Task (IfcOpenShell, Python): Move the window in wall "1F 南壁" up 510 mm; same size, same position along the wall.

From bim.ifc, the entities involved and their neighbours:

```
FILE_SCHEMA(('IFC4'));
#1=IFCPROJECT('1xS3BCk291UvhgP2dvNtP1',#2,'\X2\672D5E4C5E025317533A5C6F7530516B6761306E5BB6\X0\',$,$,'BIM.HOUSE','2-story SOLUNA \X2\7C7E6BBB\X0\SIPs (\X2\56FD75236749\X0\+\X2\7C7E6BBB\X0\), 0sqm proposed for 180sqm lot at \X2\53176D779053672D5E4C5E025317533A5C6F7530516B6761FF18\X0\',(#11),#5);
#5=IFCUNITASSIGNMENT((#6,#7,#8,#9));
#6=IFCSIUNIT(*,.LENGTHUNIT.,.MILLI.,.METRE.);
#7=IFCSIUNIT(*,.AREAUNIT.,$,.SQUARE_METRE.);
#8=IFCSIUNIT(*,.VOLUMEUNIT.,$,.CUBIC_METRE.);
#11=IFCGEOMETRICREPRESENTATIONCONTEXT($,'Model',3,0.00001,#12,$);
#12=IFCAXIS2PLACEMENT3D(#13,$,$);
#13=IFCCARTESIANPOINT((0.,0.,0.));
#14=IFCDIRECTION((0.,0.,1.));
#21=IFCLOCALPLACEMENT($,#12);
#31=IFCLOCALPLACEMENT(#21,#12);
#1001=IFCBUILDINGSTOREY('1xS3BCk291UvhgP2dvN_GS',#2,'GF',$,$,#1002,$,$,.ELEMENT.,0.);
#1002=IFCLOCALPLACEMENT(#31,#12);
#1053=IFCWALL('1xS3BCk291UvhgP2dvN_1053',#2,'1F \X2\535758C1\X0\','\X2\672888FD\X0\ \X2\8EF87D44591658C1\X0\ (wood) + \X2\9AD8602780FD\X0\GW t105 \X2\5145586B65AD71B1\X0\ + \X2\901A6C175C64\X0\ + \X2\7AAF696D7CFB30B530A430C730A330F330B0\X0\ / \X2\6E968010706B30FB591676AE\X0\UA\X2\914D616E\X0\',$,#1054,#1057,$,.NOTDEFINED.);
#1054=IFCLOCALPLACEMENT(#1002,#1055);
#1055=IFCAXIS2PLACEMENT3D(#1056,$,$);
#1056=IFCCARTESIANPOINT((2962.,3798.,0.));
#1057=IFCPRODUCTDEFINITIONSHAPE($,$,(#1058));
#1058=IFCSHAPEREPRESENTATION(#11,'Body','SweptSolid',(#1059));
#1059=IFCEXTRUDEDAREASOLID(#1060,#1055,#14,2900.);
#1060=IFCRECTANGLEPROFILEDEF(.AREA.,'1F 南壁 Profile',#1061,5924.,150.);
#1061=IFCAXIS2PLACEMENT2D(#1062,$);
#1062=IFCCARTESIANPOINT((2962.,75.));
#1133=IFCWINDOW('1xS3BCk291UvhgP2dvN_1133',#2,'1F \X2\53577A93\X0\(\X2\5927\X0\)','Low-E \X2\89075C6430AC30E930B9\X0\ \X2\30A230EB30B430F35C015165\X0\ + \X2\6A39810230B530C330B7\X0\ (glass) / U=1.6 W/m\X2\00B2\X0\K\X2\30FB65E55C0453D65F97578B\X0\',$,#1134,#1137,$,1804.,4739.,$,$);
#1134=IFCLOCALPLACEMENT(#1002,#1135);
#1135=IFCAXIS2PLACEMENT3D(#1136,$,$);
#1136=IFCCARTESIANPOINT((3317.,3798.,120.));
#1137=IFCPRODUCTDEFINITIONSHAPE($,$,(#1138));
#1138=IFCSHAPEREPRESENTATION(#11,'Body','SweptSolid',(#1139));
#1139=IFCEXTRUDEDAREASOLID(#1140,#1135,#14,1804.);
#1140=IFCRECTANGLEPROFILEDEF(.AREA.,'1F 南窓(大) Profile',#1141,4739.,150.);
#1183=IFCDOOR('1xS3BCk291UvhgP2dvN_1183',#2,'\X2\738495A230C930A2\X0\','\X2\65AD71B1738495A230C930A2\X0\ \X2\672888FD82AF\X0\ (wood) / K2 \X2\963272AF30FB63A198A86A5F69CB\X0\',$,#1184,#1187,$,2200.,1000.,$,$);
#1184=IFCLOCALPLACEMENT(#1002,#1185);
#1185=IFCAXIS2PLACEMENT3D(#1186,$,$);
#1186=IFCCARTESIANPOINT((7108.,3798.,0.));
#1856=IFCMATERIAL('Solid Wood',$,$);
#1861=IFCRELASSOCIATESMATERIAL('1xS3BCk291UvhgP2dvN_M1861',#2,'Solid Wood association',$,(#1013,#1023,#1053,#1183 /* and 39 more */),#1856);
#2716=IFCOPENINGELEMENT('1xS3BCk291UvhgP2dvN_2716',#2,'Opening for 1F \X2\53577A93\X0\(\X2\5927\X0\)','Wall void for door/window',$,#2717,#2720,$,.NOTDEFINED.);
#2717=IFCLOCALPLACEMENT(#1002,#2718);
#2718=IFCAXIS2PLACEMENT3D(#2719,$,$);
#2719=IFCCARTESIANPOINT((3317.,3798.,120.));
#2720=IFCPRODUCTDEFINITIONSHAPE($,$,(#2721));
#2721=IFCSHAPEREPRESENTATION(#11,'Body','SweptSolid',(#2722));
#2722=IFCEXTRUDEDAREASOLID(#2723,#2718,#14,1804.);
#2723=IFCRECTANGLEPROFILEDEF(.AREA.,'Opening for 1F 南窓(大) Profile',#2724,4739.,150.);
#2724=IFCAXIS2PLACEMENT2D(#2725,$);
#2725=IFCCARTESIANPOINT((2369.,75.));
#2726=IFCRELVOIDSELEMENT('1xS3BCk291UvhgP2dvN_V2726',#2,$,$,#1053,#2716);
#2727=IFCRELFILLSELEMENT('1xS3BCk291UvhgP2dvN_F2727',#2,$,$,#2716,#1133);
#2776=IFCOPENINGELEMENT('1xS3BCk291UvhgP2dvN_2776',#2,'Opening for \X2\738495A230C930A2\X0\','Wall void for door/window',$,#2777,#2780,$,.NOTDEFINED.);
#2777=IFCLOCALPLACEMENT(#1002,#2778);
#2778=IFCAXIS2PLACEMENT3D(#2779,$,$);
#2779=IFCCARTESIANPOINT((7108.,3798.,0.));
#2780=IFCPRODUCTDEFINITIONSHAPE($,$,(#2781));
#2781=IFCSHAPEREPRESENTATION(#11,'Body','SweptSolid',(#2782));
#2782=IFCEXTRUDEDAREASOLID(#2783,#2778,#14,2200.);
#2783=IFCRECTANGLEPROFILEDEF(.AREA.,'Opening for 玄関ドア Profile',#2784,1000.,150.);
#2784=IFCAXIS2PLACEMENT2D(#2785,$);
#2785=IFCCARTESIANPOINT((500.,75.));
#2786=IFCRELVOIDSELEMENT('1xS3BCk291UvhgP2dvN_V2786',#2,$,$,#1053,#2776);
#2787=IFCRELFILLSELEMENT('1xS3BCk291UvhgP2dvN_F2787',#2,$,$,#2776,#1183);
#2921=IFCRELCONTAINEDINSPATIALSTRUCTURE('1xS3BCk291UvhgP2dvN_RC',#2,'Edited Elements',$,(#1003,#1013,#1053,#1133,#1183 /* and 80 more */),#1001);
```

```python
import numpy as np
import ifcopenshell
import ifcopenshell.api.geometry
import ifcopenshell.util.placement
import ifcopenshell.util.unit

model = ifcopenshell.open("bim.ifc")
unit_scale = ifcopenshell.util.unit.calculate_unit_scale(model)

window = model.by_guid("1xS3BCk291UvhgP2dvN_1133")
opening = window.FillsVoids[0].RelatingOpeningElement
dz = 0.51 / unit_scale

shift = np.array([0.0, 0.0, dz])
# The window is not placed relative to its opening, so move both.
for product in (opening, window):
    matrix = ifcopenshell.util.placement.get_local_placement(product.ObjectPlacement)
    matrix[:3, 3] += shift
    ifcopenshell.api.geometry.edit_object_placement(model, product=product, matrix=matrix, is_si=False)

print(f"moved by {dz * unit_scale:+.3f} m")

model.write("bim_v2.ifc")
```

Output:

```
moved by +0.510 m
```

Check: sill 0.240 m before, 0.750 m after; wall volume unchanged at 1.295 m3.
